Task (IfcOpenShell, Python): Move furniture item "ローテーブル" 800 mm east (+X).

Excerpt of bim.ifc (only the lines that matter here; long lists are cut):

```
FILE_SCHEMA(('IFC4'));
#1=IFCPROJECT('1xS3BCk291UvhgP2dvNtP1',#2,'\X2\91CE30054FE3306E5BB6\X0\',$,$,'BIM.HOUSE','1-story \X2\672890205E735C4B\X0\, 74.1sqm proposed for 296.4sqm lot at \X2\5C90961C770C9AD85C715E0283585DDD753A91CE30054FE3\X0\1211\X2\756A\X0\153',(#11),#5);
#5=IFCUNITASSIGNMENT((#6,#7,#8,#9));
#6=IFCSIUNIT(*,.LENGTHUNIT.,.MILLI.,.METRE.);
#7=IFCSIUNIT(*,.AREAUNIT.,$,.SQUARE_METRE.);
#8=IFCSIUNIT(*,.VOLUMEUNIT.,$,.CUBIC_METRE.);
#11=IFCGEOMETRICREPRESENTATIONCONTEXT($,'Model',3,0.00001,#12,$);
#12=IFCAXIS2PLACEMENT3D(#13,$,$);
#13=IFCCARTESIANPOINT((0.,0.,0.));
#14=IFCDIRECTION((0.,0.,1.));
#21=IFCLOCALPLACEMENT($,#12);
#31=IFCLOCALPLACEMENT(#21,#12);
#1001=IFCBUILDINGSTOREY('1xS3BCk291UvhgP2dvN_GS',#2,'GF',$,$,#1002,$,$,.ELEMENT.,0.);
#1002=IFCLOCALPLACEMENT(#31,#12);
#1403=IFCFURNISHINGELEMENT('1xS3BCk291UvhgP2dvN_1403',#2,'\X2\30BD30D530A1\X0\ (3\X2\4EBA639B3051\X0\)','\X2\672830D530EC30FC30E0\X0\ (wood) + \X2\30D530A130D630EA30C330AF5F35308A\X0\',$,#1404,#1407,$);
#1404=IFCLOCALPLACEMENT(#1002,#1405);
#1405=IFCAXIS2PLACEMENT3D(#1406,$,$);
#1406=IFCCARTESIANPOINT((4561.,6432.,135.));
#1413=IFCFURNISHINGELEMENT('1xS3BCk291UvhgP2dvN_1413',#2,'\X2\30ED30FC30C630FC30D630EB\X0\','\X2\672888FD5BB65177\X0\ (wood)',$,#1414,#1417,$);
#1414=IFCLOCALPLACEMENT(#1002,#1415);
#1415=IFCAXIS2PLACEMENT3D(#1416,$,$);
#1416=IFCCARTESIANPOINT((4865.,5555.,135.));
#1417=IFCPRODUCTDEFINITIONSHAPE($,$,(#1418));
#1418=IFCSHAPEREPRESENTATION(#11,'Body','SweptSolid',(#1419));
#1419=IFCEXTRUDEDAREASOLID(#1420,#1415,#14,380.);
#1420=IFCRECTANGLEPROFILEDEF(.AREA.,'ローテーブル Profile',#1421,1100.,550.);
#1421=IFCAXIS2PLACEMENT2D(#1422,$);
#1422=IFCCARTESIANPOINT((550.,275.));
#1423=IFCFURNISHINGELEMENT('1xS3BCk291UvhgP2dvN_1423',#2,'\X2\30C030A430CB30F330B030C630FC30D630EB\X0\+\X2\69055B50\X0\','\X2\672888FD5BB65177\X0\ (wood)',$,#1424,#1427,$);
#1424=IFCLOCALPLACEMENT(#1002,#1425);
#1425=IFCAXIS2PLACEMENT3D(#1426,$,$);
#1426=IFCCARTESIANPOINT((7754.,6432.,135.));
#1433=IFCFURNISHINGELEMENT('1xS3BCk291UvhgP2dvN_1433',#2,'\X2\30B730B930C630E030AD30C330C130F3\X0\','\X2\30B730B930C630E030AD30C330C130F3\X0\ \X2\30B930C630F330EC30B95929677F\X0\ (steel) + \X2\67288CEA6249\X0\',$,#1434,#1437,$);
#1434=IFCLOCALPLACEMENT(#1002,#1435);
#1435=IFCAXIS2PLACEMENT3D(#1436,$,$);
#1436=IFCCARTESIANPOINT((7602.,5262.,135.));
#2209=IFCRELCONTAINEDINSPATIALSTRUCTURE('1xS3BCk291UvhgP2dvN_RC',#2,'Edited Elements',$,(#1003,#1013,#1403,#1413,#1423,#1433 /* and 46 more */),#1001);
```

```python
import ifcopenshell
import ifcopenshell.api.geometry
import ifcopenshell.util.placement

model = ifcopenshell.open("bim.ifc")

item = model.by_id(1413)
matrix = ifcopenshell.util.placement.get_local_placement(item.ObjectPlacement)
matrix[0, 3] += 800.0
ifcopenshell.api.geometry.edit_object_placement(model, product=item, matrix=matrix, is_si=False)

print(ifcopenshell.util.placement.get_local_placement(item.ObjectPlacement).round(3) + 0.0)

model.write("bim_rev.ifc")
```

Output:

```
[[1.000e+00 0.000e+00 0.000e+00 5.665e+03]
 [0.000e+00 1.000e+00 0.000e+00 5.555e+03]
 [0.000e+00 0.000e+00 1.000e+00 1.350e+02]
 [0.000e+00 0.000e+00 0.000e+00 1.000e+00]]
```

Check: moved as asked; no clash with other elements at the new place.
